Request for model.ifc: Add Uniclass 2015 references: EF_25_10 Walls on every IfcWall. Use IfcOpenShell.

First a look at what the model holds.

```python
import ifcopenshell

model = ifcopenshell.open("model.ifc")
print(model.schema)
print("classifications:", [c.Name for c in model.by_type("IfcClassification")])
for ifc_class in ("IfcDoor", "IfcRoof", "IfcStair", "IfcWall", "IfcWindow"):
    print(ifc_class, len(model.by_type(ifc_class)))
```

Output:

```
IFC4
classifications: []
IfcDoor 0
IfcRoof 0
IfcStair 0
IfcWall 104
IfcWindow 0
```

```python
import ifcopenshell
import ifcopenshell.api.classification

model = ifcopenshell.open("model.ifc")

system = ifcopenshell.api.classification.add_classification(model, classification="Uniclass 2015")

codes = {
    "IfcWall": ("EF_25_10", "Walls"),
}
for ifc_class, (code, name) in codes.items():
    products = model.by_type(ifc_class)
    ifcopenshell.api.classification.add_reference(
        model, products=products, classification=system, identification=code, name=name
    )
    print(code, len(products))

model.write("model_rev.ifc")
```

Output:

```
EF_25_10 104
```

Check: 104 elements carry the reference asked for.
